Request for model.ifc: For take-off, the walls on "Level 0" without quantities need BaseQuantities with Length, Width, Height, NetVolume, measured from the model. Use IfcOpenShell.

First a look at what the model holds.

```python
import ifcopenshell
import ifcopenshell.util.element
import ifcopenshell.util.unit

model = ifcopenshell.open("model.ifc")
print(model.schema)
for unit_type in ("LENGTHUNIT", "AREAUNIT", "VOLUMEUNIT"):
    print(unit_type, ifcopenshell.util.unit.calculate_unit_scale(model, unit_type))
storey = next(s for s in model.by_type("IfcBuildingStorey") if s.Name == "Level 0")
walls = [e for e in ifcopenshell.util.element.get_decomposition(storey) if e.is_a("IfcWall")]
for e in sorted(walls, key=lambda e: e.id()):
    print(e.id(), e.is_a(), e.Name, list(ifcopenshell.util.element.get_psets(e, qtos_only=True)), sep=" | ")
```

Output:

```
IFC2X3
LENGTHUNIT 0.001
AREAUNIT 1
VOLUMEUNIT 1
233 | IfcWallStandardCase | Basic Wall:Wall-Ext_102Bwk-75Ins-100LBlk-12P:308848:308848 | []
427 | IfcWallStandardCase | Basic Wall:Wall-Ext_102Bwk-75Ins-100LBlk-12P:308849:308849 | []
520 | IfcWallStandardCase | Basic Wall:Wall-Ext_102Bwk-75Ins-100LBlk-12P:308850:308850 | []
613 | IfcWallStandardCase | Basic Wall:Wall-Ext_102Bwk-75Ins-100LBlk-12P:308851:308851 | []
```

```python
import ifcopenshell
import ifcopenshell.api.pset
import ifcopenshell.geom
import ifcopenshell.util.element
import ifcopenshell.util.shape
import ifcopenshell.util.unit

model = ifcopenshell.open("model.ifc")
unit_scale = ifcopenshell.util.unit.calculate_unit_scale(model)
volume_scale = ifcopenshell.util.unit.calculate_unit_scale(model, "VOLUMEUNIT")
settings = ifcopenshell.geom.settings()

storey = next(s for s in model.by_type("IfcBuildingStorey") if s.Name == "Level 0")
walls = [e for e in ifcopenshell.util.element.get_decomposition(storey) if e.is_a("IfcWall")]

for e in sorted(walls, key=lambda e: e.id()):
    if ifcopenshell.util.element.get_psets(e, qtos_only=True, should_inherit=False):
        continue
    # Geometry comes back in metres, in the element's own axes.
    shape = ifcopenshell.geom.create_shape(settings, e)
    values = {
        "Length": ifcopenshell.util.shape.get_x(shape.geometry) / unit_scale,
        "Width": ifcopenshell.util.shape.get_y(shape.geometry) / unit_scale,
        "Height": ifcopenshell.util.shape.get_z(shape.geometry) / unit_scale,
        "NetVolume": ifcopenshell.util.shape.get_volume(shape.geometry) / volume_scale,
    }
    qto = ifcopenshell.api.pset.add_qto(model, product=e, name="BaseQuantities")
    ifcopenshell.api.pset.edit_qto(model, qto=qto, properties=values)
    print(e.id(), {k: round(v, 3) for k, v in values.items()})

model.write("model-out.ifc")
```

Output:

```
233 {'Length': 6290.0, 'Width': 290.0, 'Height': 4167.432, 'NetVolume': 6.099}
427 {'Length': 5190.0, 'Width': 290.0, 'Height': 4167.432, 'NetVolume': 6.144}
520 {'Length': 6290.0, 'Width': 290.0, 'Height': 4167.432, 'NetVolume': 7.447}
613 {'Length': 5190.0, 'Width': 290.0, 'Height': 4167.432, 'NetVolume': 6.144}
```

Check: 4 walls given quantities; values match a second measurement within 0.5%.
